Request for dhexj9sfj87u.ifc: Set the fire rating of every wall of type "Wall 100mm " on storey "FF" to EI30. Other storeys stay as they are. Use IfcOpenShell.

First a look at what the model holds.

```python
import ifcopenshell
import ifcopenshell.util.element

model = ifcopenshell.open("dhexj9sfj87u.ifc")
print(model.schema)
storey = next(s for s in model.by_type("IfcBuildingStorey") if s.Name == "FF")
walls = [e for e in ifcopenshell.util.element.get_decomposition(storey) if e.is_a("IfcWall")]
seen = {}
for e in walls:
    element_type = ifcopenshell.util.element.get_type(e)
    key = (element_type.Name if element_type != e and element_type else None, ifcopenshell.util.element.get_pset(e, "Pset_WallCommon", "FireRating"))
    seen[key] = seen.get(key, 0) + 1
for (name, value), count in sorted(seen.items(), key=str):
    print(count, "x", name, "|", value)
```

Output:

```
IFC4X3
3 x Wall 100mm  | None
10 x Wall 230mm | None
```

```python
import ifcopenshell
import ifcopenshell.api.pset
import ifcopenshell.util.element

model = ifcopenshell.open("dhexj9sfj87u.ifc")

storey = next(s for s in model.by_type("IfcBuildingStorey") if s.Name == "FF")
walls = [e for e in ifcopenshell.util.element.get_decomposition(storey) if e.is_a("IfcWall")]

count = 0
for e in walls:
    element_type = ifcopenshell.util.element.get_type(e)
    if element_type in (None, e) or element_type.Name != "Wall 100mm ":
        continue
    # add_pset returns the element's existing set when there is one.
    pset = ifcopenshell.api.pset.add_pset(model, product=e, name="Pset_WallCommon")
    ifcopenshell.api.pset.edit_pset(model, pset=pset, properties={"FireRating": "EI30"})
    count += 1

print(count, "walls updated")

model.write("dhexj9sfj87u-out.ifc")
```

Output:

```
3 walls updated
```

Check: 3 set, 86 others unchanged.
